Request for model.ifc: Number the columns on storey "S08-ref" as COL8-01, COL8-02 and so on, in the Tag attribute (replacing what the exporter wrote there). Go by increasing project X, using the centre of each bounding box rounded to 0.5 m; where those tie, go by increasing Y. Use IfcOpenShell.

First a look at what the model holds.

```python
import ifcopenshell
import ifcopenshell.util.element
import ifcopenshell.util.placement

model = ifcopenshell.open("model.ifc")
print(model.schema)
storey = next(s for s in model.by_type("IfcBuildingStorey") if s.Name == "S08-ref")
columns = [e for e in ifcopenshell.util.element.get_decomposition(storey) if e.is_a("IfcColumn")]
for e in sorted(columns, key=lambda e: e.id()):
    origin = ifcopenshell.util.placement.get_local_placement(e.ObjectPlacement)[:3, 3]
    print(e.id(), e.Tag, e.Name, origin.round(2) + 0.0, sep=" | ")
```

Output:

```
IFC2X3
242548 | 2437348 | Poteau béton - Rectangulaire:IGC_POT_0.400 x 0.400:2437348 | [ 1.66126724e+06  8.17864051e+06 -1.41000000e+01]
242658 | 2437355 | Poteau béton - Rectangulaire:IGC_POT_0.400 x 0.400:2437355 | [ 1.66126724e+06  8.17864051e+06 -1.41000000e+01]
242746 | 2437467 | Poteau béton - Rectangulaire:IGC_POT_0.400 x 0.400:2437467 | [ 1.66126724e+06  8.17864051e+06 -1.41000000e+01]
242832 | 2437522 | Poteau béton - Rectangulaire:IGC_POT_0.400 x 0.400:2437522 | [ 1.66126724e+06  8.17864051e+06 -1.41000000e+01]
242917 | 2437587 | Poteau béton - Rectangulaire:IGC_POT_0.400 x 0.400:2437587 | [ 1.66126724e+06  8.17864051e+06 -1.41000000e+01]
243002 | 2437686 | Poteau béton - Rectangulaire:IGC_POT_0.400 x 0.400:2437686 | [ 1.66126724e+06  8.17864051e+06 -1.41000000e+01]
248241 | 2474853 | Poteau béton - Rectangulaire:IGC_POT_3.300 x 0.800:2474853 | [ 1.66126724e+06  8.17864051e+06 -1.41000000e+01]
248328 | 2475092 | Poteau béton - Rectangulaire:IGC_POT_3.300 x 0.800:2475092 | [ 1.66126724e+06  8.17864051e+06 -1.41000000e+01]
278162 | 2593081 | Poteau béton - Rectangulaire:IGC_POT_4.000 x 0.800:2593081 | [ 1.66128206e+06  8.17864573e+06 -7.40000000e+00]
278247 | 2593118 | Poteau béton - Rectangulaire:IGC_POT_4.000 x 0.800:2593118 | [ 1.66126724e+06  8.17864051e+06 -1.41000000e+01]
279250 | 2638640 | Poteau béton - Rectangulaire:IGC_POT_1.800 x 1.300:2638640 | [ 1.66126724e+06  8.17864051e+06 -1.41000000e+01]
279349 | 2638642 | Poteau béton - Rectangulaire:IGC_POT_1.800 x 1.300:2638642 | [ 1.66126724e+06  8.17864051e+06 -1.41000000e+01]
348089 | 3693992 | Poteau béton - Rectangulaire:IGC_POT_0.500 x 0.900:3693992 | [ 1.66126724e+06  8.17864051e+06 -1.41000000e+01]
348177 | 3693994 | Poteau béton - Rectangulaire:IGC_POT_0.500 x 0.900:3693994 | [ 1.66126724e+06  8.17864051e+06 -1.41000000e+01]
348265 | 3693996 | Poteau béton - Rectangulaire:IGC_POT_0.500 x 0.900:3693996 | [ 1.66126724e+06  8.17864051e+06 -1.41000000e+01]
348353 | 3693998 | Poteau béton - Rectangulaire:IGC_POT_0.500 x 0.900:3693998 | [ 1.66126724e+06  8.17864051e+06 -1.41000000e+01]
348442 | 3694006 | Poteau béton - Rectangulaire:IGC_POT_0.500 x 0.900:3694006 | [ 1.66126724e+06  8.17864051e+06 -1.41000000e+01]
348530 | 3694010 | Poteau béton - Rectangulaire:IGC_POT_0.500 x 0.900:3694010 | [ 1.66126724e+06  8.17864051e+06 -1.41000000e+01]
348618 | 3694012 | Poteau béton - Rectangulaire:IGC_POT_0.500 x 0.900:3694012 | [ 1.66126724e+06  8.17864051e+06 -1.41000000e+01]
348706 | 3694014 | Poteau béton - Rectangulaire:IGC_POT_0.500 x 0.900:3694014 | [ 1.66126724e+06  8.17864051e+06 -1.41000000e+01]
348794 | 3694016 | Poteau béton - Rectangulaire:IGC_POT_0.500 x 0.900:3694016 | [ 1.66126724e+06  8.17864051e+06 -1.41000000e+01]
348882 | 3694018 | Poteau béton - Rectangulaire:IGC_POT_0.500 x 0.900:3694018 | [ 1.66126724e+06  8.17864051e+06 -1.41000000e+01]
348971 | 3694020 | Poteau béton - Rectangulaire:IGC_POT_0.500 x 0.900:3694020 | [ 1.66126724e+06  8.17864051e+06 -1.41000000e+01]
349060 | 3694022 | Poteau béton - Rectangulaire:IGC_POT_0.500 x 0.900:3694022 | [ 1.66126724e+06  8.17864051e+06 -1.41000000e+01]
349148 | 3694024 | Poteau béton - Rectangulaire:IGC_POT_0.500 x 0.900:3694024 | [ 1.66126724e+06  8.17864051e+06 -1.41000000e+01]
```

```python
import ifcopenshell
import ifcopenshell.geom
import ifcopenshell.util.element
import ifcopenshell.util.shape

model = ifcopenshell.open("model.ifc")
settings = ifcopenshell.geom.settings()
settings.set("use-world-coords", True)


def centre(element):
    shape = ifcopenshell.geom.create_shape(settings, element)
    return ifcopenshell.util.shape.get_bbox_centroid(shape.geometry)


storey = next(s for s in model.by_type("IfcBuildingStorey") if s.Name == "S08-ref")
columns = [e for e in ifcopenshell.util.element.get_decomposition(storey) if e.is_a("IfcColumn")]

# Insertion points can sit at a corner or the storey origin, so sort by the geometry (in metres).
centres = {e: centre(e) for e in columns}
columns.sort(key=lambda e: (round(centres[e][0] / 0.5), centres[e][1]))

for i, e in enumerate(columns, start=1):
    number = f"COL8-{i:02d}"
    e.Tag = number
    print(e.id(), number)

model.write("model_v2.ifc")
```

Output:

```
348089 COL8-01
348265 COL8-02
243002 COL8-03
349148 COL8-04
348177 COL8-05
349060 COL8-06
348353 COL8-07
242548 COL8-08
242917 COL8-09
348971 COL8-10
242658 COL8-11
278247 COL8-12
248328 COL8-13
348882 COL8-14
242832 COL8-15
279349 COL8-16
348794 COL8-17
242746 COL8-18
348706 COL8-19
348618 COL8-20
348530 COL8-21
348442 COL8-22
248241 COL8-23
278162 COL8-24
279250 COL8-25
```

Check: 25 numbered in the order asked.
